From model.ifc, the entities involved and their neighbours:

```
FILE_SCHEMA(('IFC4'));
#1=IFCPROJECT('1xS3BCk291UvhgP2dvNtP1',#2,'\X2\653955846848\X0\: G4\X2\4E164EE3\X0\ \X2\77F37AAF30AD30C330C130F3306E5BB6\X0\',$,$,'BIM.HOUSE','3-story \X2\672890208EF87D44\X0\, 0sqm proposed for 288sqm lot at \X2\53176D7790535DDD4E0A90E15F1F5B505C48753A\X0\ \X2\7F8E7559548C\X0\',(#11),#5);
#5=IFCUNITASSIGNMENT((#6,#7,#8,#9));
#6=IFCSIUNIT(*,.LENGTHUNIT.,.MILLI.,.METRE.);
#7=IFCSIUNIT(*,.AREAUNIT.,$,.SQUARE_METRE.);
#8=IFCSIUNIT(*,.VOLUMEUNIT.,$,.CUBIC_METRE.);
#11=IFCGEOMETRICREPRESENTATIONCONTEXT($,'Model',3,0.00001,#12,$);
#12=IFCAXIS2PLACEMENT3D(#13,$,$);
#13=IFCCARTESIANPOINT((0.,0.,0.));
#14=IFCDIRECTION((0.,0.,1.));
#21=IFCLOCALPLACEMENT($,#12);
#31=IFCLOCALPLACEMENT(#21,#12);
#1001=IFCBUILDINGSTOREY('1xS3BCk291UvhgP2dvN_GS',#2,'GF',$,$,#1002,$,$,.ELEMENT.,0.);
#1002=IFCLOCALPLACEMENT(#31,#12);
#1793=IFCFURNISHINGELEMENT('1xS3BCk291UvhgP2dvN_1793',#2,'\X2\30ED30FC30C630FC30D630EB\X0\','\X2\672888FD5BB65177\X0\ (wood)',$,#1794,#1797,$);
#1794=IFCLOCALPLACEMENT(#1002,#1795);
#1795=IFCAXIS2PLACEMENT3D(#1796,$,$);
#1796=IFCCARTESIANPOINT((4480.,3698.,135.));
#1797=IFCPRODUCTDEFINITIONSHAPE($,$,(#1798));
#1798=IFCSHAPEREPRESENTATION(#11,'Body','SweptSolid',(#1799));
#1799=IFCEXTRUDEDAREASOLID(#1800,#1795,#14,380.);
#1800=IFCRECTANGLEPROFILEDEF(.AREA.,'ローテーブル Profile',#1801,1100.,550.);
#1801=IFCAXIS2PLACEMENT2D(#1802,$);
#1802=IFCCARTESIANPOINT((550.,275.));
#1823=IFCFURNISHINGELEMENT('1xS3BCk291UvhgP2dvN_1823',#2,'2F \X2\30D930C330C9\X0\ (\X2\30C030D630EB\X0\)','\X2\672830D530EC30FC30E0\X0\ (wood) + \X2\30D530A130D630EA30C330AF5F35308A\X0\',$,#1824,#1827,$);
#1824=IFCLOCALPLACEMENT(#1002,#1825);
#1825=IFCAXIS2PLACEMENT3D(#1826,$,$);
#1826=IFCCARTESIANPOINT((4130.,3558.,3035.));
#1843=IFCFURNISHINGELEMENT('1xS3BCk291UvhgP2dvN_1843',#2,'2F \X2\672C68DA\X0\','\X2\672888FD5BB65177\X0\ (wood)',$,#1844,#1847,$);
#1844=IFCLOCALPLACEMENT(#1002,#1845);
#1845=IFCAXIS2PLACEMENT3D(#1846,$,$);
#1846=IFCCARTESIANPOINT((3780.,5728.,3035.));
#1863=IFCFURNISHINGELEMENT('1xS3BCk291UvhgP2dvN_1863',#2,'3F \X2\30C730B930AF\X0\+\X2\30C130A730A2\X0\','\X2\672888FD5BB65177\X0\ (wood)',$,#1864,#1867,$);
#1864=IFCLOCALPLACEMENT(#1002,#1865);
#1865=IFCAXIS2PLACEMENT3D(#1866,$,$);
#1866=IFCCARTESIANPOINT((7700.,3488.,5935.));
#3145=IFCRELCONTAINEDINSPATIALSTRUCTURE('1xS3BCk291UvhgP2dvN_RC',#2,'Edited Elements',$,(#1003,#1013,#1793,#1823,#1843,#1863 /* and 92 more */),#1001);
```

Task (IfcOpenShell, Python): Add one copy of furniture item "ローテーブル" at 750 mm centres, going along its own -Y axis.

```python
import ifcopenshell
import ifcopenshell.api.geometry
import ifcopenshell.api.root
import ifcopenshell.util.element
import ifcopenshell.util.placement
import ifcopenshell.util.unit

model = ifcopenshell.open("model.ifc")
unit_scale = ifcopenshell.util.unit.calculate_unit_scale(model)


def reuse_history(source, copy):
    """copy_class also copies each property set's owner history, people and application; keep the originals."""
    for rel in copy.IsDefinedBy:
        if rel.is_a("IfcRelDefinesByProperties") and (history := rel.RelatingPropertyDefinition.OwnerHistory):
            rel.RelatingPropertyDefinition.OwnerHistory = source.OwnerHistory
            ifcopenshell.util.element.remove_deep2(model, history)


source = model.by_id(1793)
base = ifcopenshell.util.placement.get_local_placement(source.ObjectPlacement)
step = -base[:3, 1] * 0.75 / unit_scale

for i in range(1, 2):
    copy = ifcopenshell.api.root.copy_class(model, product=source)
    copy.Representation = ifcopenshell.util.element.copy_deep(
        model, source.Representation, exclude=["IfcGeometricRepresentationContext", "IfcRepresentationMap"]
    )
    reuse_history(source, copy)
    matrix = base.copy()
    matrix[:3, 3] += i * step
    print("added at", matrix[:3, 3].round(3) + 0.0)
    ifcopenshell.api.geometry.edit_object_placement(model, product=copy, matrix=matrix, is_si=False)

model.write("model_updated.ifc")
```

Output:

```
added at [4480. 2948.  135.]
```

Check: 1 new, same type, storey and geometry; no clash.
